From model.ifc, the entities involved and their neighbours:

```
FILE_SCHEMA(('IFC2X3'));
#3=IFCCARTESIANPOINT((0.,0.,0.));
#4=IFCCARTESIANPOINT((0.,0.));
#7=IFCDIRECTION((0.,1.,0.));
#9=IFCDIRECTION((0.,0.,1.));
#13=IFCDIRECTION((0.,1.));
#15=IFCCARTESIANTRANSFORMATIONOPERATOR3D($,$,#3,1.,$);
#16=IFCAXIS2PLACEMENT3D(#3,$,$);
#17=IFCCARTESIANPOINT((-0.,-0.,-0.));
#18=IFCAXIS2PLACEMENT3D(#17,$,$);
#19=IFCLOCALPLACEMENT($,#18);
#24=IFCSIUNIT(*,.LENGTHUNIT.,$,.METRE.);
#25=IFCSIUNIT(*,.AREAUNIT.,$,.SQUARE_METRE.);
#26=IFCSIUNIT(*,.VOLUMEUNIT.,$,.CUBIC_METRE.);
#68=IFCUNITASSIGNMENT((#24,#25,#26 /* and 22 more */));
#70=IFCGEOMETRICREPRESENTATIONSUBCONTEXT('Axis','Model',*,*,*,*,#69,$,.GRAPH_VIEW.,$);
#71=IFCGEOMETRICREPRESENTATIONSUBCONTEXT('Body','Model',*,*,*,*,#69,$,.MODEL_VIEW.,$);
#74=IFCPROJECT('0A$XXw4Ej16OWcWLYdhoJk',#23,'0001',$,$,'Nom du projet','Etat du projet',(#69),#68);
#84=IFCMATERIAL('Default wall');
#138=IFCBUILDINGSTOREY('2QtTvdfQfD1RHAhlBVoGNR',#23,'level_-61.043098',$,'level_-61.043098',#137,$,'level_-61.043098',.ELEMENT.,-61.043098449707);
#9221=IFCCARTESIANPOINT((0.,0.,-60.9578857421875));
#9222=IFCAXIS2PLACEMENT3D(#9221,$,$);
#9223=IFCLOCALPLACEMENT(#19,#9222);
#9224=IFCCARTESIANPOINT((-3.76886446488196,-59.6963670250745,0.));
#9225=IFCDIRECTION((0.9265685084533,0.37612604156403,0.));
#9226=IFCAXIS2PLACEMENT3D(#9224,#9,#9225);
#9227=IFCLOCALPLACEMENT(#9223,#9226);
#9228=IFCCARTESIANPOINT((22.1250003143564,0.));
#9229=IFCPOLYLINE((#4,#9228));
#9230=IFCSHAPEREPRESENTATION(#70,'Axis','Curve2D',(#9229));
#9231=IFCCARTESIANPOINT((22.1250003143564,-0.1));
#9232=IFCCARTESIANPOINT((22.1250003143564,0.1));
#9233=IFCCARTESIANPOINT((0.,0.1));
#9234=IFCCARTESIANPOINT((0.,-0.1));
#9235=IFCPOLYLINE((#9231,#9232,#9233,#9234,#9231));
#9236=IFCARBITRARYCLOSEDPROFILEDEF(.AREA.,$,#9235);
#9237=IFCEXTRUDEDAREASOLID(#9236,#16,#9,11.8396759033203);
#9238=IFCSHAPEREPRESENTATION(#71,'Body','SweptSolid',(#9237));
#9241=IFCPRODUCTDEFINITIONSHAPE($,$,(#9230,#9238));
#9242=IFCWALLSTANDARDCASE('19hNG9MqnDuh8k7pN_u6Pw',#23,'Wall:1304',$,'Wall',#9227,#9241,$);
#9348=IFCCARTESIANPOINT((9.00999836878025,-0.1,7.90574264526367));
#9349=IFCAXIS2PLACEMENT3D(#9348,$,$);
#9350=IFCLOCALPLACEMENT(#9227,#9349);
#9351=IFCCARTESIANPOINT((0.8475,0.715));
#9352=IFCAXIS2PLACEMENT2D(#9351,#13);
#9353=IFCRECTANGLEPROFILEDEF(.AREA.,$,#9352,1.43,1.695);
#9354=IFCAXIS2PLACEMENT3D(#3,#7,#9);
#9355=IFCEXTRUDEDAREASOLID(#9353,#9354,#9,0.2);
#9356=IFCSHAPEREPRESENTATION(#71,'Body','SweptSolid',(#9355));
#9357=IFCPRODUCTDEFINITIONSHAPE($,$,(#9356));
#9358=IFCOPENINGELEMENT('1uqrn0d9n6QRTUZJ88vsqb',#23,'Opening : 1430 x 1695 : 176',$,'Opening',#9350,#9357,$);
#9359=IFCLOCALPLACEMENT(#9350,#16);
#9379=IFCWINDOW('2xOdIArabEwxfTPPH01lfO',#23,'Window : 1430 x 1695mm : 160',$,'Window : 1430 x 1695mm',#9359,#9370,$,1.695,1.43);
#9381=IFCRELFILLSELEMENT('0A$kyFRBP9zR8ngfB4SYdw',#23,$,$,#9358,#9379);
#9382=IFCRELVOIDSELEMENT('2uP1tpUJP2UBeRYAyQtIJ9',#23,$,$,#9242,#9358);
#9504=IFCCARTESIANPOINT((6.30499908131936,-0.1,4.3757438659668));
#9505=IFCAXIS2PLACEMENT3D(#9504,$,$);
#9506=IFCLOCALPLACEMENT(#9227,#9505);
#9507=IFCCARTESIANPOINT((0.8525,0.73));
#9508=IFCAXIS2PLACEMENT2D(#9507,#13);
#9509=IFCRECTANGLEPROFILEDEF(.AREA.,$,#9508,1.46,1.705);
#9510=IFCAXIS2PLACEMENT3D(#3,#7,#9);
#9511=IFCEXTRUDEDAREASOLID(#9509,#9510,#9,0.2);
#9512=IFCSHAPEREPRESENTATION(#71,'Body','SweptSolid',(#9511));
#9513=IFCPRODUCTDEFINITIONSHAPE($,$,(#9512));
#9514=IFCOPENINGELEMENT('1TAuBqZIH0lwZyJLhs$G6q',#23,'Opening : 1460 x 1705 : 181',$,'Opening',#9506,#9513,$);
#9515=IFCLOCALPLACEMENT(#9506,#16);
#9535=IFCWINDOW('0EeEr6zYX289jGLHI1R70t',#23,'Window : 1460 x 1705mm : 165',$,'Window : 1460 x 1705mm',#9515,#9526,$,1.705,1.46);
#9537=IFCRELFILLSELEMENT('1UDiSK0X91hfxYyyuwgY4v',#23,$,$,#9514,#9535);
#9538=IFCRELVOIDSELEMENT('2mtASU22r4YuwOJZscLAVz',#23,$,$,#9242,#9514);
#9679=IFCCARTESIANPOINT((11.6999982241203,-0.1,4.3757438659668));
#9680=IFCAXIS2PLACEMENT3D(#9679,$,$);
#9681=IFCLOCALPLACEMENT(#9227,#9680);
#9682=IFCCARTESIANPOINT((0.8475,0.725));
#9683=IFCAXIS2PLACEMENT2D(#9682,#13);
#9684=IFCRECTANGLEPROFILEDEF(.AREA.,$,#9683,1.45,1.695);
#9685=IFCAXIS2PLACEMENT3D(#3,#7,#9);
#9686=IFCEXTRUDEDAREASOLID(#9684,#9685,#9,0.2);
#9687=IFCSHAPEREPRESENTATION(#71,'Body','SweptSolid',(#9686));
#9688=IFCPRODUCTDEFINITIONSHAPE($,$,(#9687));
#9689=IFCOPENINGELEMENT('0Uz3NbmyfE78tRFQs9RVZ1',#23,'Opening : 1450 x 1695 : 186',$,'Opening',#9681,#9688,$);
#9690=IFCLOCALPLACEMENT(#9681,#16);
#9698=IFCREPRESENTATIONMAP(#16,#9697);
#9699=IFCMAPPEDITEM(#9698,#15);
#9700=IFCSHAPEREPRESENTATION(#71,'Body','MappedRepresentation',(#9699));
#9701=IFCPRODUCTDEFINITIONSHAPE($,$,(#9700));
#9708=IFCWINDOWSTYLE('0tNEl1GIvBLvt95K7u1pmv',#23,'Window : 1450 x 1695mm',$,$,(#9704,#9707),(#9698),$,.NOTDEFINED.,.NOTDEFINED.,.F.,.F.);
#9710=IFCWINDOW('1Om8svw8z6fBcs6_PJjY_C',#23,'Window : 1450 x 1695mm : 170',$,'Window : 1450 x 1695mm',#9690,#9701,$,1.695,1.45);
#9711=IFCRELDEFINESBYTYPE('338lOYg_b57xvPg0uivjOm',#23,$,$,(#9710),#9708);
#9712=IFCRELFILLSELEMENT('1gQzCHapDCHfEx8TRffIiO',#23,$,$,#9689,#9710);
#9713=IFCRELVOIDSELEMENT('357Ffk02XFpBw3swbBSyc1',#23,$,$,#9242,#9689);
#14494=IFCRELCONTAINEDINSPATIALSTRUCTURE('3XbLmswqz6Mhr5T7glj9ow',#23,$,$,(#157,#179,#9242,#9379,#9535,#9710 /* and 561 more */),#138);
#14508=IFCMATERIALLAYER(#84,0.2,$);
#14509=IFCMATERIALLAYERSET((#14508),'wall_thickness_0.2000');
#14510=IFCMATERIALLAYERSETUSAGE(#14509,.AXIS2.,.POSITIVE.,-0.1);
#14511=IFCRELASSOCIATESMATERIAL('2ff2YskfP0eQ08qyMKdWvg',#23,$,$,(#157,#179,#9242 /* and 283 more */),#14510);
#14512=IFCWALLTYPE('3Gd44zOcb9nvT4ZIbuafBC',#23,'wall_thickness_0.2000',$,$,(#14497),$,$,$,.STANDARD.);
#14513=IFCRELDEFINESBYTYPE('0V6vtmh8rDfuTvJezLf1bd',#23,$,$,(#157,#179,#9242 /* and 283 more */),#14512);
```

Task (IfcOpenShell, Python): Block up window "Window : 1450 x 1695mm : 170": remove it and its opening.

```python
import ifcopenshell
import ifcopenshell.api.feature
import ifcopenshell.api.root
import ifcopenshell.geom
import ifcopenshell.util.shape

model = ifcopenshell.open("model.ifc")
settings = ifcopenshell.geom.settings()


def volume(element):
    """Net volume in cubic metres, openings subtracted."""
    shape = ifcopenshell.geom.create_shape(settings, element)
    return ifcopenshell.util.shape.get_volume(shape.geometry)


window = model.by_id(9710)
opening = window.FillsVoids[0].RelatingOpeningElement
wall = opening.VoidsElements[0].RelatingBuildingElement
before = volume(wall)

ifcopenshell.api.root.remove_product(model, product=window)
ifcopenshell.api.feature.remove_feature(model, feature=opening)

after = volume(wall)

print(f"wall volume {before:.3f} -> {after:.3f} m3")

model.write("model_v2.ifc")
```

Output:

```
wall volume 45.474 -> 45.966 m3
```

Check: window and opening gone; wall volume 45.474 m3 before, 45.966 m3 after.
